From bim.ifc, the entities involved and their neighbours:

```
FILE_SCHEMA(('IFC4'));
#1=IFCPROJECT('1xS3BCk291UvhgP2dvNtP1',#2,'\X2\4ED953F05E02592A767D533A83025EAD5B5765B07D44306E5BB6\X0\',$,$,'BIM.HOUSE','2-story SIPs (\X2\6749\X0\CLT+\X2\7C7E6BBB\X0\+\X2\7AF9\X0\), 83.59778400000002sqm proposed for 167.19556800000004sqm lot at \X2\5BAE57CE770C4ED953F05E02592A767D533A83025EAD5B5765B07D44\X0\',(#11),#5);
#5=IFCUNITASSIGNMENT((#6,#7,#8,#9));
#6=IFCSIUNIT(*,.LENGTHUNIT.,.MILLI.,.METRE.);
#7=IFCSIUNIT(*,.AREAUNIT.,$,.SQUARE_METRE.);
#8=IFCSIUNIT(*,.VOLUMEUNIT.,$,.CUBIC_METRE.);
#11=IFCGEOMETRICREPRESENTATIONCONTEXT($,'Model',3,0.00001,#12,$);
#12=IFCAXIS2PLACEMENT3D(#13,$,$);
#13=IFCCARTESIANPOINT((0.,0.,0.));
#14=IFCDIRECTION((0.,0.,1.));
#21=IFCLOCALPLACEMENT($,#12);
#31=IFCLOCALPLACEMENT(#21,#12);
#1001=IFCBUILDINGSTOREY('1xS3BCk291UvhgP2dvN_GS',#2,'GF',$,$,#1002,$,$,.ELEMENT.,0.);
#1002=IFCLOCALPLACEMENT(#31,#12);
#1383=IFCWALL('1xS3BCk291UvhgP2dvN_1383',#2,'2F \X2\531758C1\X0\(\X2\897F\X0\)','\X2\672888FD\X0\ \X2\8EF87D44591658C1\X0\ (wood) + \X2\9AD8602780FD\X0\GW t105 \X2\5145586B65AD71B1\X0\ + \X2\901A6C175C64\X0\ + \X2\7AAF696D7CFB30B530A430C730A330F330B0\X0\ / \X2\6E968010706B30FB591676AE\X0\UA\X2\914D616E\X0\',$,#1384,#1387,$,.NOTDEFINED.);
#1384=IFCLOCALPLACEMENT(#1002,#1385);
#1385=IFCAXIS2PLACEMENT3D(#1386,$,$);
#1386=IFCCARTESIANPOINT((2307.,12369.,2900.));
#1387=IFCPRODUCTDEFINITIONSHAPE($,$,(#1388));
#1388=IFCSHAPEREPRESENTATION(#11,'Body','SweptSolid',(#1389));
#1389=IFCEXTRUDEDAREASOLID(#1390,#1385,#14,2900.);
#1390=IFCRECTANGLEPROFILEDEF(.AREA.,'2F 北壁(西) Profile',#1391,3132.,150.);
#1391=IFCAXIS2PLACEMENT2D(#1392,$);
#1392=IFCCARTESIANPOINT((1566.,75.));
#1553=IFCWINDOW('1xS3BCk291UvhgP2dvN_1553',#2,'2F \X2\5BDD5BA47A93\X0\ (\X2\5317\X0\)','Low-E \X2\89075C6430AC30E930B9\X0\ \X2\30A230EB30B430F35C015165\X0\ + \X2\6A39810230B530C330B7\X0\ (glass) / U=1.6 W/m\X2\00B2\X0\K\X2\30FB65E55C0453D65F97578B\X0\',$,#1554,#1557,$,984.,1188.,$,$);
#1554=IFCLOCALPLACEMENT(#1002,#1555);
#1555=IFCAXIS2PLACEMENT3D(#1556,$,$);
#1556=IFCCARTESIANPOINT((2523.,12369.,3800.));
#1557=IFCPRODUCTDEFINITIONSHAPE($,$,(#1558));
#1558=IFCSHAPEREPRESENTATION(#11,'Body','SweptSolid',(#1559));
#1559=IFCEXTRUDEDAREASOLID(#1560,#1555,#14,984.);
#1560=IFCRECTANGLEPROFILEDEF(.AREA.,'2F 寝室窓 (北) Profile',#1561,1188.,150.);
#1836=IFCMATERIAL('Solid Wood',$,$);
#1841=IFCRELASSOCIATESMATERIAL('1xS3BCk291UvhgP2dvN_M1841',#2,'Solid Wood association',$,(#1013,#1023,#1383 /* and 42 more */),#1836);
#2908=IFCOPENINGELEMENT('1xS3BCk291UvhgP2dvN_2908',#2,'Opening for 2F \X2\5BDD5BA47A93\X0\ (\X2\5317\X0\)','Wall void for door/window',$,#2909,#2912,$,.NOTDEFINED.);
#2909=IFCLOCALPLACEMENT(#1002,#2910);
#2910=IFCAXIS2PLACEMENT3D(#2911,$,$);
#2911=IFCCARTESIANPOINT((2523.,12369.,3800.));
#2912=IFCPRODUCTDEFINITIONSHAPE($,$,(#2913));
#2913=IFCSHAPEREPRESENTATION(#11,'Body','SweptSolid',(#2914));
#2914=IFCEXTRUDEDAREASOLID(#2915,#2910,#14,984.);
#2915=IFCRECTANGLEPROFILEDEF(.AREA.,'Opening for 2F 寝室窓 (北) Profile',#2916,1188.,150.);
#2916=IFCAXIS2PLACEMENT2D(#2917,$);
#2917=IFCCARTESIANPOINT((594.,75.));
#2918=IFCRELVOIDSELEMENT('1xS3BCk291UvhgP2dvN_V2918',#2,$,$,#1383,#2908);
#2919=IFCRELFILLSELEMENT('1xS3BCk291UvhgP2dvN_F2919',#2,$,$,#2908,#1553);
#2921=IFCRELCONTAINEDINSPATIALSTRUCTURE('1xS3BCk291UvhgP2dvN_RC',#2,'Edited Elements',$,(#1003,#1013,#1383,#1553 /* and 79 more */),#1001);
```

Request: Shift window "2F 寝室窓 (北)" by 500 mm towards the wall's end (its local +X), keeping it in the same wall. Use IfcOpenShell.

```python
import ifcopenshell
import ifcopenshell.api.geometry
import ifcopenshell.util.placement
import ifcopenshell.util.unit

model = ifcopenshell.open("bim.ifc")
unit_scale = ifcopenshell.util.unit.calculate_unit_scale(model)

window = model.by_id(1553)
opening = window.FillsVoids[0].RelatingOpeningElement
wall = opening.VoidsElements[0].RelatingBuildingElement

wall_matrix = ifcopenshell.util.placement.get_local_placement(wall.ObjectPlacement)
shift = wall_matrix[:3, 0] * 0.5 / unit_scale
before = ifcopenshell.util.placement.get_local_placement(window.ObjectPlacement)[:3, 3].copy()

# The window is not placed relative to its opening, so move both.
for product in (opening, window):
    matrix = ifcopenshell.util.placement.get_local_placement(product.ObjectPlacement)
    matrix[:3, 3] += shift
    ifcopenshell.api.geometry.edit_object_placement(model, product=product, matrix=matrix, is_si=False)

after = ifcopenshell.util.placement.get_local_placement(window.ObjectPlacement)[:3, 3]
print("window moved by", (after - before).round(3) + 0.0)

model.write("bim_rev.ifc")
```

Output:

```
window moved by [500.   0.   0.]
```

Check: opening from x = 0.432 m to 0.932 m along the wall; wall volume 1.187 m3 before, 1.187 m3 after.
